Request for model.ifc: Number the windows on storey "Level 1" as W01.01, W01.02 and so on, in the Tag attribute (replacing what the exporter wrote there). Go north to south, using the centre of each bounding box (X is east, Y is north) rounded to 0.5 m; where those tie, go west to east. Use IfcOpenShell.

First a look at what the model holds.

```python
import ifcopenshell
import ifcopenshell.util.element
import ifcopenshell.util.placement

model = ifcopenshell.open("model.ifc")
print(model.schema)
storey = next(s for s in model.by_type("IfcBuildingStorey") if s.Name == "Level 1")
windows = [e for e in ifcopenshell.util.element.get_decomposition(storey) if e.is_a("IfcWindow")]
for e in sorted(windows, key=lambda e: e.id()):
    origin = ifcopenshell.util.placement.get_local_placement(e.ObjectPlacement)[:3, 3]
    print(e.id(), e.Tag, e.Name, origin.round(2) + 0.0, sep=" | ")
```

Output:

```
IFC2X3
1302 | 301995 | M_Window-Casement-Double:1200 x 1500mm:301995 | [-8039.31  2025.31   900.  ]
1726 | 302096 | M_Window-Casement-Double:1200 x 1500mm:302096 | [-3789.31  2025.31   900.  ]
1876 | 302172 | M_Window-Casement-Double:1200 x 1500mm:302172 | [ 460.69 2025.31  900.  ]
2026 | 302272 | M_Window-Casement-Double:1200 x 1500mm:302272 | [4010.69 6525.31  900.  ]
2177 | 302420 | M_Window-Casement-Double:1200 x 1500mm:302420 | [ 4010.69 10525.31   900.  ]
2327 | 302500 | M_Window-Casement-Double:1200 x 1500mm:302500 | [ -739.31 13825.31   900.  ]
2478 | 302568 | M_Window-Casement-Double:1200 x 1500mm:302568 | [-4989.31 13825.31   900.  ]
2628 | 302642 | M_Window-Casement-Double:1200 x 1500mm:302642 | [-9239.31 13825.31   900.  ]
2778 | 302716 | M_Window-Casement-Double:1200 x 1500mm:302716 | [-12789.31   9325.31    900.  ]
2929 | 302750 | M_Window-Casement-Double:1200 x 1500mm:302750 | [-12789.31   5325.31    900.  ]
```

```python
import ifcopenshell
import ifcopenshell.geom
import ifcopenshell.util.element
import ifcopenshell.util.shape

model = ifcopenshell.open("model.ifc")
settings = ifcopenshell.geom.settings()
settings.set("use-world-coords", True)


def centre(element):
    shape = ifcopenshell.geom.create_shape(settings, element)
    return ifcopenshell.util.shape.get_bbox_centroid(shape.geometry)


storey = next(s for s in model.by_type("IfcBuildingStorey") if s.Name == "Level 1")
windows = [e for e in ifcopenshell.util.element.get_decomposition(storey) if e.is_a("IfcWindow")]

# Insertion points can sit at a corner or the storey origin, so sort by the geometry (in metres).
centres = {e: centre(e) for e in windows}
windows.sort(key=lambda e: (-round(centres[e][1] / 0.5), centres[e][0]))

for i, e in enumerate(windows, start=1):
    number = f"W01.{i:02d}"
    e.Tag = number
    print(e.id(), number)

model.write("model_updated.ifc")
```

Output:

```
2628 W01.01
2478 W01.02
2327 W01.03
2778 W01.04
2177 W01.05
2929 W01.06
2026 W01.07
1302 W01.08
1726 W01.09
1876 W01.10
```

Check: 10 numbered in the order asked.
